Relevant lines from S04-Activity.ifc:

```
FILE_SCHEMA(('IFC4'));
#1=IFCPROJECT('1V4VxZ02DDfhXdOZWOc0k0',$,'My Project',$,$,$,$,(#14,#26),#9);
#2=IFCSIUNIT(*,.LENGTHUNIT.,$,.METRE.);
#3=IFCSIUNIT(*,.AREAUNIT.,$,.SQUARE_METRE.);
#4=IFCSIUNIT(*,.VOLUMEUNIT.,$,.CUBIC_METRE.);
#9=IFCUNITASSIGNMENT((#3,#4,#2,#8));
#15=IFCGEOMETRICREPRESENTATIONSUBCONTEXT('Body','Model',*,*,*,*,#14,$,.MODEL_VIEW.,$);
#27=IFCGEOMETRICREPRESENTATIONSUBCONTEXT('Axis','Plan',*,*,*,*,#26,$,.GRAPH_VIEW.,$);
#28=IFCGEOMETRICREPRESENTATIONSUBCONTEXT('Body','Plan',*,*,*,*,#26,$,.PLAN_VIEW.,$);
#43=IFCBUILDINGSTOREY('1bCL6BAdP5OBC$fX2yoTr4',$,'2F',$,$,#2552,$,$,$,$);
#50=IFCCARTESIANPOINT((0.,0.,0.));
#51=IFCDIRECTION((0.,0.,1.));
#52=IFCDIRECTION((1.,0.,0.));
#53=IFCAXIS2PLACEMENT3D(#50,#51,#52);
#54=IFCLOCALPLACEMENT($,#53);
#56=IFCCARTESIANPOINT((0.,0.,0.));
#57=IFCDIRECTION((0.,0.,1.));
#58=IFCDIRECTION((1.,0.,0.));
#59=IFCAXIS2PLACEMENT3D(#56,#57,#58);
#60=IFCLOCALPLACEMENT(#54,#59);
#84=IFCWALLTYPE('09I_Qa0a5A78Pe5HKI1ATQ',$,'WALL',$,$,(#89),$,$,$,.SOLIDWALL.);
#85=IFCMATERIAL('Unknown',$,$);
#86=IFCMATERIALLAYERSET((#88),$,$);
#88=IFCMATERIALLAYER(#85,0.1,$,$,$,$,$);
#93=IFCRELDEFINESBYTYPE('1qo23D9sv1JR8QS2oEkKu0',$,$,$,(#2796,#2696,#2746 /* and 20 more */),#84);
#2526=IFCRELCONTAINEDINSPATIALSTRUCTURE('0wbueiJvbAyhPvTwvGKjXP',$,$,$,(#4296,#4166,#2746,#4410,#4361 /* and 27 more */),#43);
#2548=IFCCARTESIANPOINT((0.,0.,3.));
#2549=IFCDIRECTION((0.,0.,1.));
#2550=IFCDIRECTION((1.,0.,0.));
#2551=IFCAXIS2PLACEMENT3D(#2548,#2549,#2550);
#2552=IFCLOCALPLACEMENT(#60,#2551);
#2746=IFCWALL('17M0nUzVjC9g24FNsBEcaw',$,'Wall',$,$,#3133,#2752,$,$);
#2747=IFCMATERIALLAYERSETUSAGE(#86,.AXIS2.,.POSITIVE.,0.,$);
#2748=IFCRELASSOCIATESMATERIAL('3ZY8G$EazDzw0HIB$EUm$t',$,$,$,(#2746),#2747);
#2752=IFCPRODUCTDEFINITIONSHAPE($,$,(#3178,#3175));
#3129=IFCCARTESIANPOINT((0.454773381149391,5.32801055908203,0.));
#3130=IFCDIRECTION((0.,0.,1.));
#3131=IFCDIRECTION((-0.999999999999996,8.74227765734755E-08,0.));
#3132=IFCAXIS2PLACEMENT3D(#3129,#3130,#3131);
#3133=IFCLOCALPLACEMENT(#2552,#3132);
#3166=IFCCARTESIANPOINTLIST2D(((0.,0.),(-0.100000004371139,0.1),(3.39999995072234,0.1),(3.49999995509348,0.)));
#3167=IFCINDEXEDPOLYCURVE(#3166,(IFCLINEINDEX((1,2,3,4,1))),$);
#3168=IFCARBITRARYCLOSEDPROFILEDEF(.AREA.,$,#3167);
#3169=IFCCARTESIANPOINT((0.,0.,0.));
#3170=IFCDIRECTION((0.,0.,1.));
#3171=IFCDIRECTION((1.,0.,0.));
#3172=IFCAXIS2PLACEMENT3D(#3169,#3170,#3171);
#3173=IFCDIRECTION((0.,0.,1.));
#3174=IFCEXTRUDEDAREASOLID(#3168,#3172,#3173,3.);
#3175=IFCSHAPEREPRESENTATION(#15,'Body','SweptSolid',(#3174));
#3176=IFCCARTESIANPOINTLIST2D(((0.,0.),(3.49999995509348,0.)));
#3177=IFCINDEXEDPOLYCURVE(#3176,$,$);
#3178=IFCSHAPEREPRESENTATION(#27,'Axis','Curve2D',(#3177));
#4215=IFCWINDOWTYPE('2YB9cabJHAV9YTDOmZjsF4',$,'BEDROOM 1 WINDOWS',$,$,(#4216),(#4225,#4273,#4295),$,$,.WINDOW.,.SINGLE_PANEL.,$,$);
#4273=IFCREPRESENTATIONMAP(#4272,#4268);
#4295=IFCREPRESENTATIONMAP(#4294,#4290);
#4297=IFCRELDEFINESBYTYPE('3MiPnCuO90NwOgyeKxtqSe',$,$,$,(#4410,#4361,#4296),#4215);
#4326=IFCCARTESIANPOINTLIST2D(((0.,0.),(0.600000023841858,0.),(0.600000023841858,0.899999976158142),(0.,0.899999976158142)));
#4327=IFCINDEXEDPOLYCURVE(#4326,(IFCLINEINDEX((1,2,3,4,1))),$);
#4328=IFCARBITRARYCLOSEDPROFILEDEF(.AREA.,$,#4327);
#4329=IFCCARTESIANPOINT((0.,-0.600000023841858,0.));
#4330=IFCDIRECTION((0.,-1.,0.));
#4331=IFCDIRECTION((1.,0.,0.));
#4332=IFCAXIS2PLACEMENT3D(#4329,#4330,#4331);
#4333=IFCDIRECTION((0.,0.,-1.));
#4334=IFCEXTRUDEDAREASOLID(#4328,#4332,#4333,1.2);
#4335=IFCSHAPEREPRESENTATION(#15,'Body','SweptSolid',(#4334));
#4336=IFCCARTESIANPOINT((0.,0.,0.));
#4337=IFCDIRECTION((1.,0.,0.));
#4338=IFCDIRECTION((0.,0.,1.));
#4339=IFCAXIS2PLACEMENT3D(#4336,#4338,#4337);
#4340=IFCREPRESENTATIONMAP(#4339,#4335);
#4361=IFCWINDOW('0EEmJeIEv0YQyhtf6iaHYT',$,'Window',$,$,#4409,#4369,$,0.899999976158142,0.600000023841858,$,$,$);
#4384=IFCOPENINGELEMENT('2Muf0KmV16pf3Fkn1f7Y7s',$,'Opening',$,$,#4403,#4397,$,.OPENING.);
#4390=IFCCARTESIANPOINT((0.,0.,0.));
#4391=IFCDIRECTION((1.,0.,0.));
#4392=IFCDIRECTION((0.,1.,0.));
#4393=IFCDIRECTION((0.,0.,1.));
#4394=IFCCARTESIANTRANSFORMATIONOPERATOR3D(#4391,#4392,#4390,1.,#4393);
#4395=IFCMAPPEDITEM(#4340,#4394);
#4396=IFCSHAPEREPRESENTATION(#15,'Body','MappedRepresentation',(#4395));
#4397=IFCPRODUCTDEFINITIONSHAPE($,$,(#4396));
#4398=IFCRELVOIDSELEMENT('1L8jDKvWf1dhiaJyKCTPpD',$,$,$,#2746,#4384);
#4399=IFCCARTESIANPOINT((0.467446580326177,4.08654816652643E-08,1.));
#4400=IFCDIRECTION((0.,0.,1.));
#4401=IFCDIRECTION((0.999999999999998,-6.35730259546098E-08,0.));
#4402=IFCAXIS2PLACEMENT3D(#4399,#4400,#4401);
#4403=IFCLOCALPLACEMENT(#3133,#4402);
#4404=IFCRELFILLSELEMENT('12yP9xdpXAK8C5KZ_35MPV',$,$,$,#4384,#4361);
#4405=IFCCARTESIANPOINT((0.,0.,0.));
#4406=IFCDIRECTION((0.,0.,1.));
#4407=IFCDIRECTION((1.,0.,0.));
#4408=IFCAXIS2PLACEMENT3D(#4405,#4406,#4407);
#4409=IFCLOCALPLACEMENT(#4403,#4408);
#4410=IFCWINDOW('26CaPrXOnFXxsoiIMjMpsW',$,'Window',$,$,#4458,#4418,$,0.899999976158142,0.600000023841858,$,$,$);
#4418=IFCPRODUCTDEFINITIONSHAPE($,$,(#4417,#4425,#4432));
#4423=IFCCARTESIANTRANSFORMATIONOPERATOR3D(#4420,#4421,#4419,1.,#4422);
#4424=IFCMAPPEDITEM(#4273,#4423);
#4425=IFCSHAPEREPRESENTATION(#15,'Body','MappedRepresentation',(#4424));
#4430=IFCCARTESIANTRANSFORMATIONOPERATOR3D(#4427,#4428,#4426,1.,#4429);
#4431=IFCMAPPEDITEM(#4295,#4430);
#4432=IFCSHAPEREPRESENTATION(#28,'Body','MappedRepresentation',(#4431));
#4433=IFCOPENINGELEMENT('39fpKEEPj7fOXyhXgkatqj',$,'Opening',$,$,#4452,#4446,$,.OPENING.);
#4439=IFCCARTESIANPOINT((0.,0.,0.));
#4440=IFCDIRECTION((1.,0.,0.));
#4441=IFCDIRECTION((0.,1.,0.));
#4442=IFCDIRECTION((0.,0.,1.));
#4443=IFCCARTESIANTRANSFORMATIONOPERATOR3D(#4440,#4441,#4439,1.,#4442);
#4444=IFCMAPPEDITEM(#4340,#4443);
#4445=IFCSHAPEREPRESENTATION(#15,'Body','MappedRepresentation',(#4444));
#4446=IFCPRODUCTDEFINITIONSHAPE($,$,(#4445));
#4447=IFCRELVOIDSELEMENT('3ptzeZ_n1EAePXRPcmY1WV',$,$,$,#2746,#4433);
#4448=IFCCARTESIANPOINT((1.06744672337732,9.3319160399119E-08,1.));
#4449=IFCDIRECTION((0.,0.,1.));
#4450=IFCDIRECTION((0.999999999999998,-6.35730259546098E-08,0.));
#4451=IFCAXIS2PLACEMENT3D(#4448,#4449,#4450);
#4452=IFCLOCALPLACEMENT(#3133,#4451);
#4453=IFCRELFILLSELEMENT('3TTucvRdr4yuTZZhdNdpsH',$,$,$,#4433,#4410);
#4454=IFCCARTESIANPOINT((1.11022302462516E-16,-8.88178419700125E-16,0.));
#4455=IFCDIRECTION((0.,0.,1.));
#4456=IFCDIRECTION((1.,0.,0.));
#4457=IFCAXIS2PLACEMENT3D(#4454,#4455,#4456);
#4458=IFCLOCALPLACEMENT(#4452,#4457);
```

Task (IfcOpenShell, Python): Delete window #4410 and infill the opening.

```python
import ifcopenshell
import ifcopenshell.api.feature
import ifcopenshell.api.root
import ifcopenshell.geom
import ifcopenshell.util.shape

model = ifcopenshell.open("S04-Activity.ifc")
settings = ifcopenshell.geom.settings()


def volume(element):
    """Net volume in cubic metres, openings subtracted."""
    shape = ifcopenshell.geom.create_shape(settings, element)
    return ifcopenshell.util.shape.get_volume(shape.geometry)


window = model.by_guid("26CaPrXOnFXxsoiIMjMpsW")
opening = window.FillsVoids[0].RelatingOpeningElement
wall = opening.VoidsElements[0].RelatingBuildingElement
before = volume(wall)

ifcopenshell.api.root.remove_product(model, product=window)
ifcopenshell.api.feature.remove_feature(model, feature=opening)

after = volume(wall)

print(f"wall volume {before:.3f} -> {after:.3f} m3")

model.write("S04-Activity-out.ifc")
```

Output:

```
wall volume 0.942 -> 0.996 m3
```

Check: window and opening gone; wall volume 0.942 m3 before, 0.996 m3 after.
